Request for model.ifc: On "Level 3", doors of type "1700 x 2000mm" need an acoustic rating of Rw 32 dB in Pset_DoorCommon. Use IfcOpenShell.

First a look at what the model holds.

```python
import ifcopenshell
import ifcopenshell.util.element

model = ifcopenshell.open("model.ifc")
print(model.schema)
storey = next(s for s in model.by_type("IfcBuildingStorey") if s.Name == "Level 3")
doors = [e for e in ifcopenshell.util.element.get_decomposition(storey) if e.is_a("IfcDoor")]
seen = {}
for e in doors:
    element_type = ifcopenshell.util.element.get_type(e)
    key = (element_type.Name if element_type != e and element_type else None, ifcopenshell.util.element.get_pset(e, "Pset_DoorCommon", "AcousticRating"))
    seen[key] = seen.get(key, 0) + 1
for (name, value), count in sorted(seen.items(), key=str):
    print(count, "x", name, "|", value)
```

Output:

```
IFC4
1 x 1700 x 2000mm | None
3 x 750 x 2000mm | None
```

```python
import ifcopenshell
import ifcopenshell.api.pset
import ifcopenshell.util.element

model = ifcopenshell.open("model.ifc")

storey = next(s for s in model.by_type("IfcBuildingStorey") if s.Name == "Level 3")
doors = [e for e in ifcopenshell.util.element.get_decomposition(storey) if e.is_a("IfcDoor")]

count = 0
for e in doors:
    element_type = ifcopenshell.util.element.get_type(e)
    if element_type in (None, e) or element_type.Name != "1700 x 2000mm":
        continue
    # add_pset returns the element's existing set when there is one.
    pset = ifcopenshell.api.pset.add_pset(model, product=e, name="Pset_DoorCommon")
    ifcopenshell.api.pset.edit_pset(model, pset=pset, properties={"AcousticRating": "Rw 32 dB"})
    count += 1

print(count, "doors updated")

model.write("model_updated.ifc")
```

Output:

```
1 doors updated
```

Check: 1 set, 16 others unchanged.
